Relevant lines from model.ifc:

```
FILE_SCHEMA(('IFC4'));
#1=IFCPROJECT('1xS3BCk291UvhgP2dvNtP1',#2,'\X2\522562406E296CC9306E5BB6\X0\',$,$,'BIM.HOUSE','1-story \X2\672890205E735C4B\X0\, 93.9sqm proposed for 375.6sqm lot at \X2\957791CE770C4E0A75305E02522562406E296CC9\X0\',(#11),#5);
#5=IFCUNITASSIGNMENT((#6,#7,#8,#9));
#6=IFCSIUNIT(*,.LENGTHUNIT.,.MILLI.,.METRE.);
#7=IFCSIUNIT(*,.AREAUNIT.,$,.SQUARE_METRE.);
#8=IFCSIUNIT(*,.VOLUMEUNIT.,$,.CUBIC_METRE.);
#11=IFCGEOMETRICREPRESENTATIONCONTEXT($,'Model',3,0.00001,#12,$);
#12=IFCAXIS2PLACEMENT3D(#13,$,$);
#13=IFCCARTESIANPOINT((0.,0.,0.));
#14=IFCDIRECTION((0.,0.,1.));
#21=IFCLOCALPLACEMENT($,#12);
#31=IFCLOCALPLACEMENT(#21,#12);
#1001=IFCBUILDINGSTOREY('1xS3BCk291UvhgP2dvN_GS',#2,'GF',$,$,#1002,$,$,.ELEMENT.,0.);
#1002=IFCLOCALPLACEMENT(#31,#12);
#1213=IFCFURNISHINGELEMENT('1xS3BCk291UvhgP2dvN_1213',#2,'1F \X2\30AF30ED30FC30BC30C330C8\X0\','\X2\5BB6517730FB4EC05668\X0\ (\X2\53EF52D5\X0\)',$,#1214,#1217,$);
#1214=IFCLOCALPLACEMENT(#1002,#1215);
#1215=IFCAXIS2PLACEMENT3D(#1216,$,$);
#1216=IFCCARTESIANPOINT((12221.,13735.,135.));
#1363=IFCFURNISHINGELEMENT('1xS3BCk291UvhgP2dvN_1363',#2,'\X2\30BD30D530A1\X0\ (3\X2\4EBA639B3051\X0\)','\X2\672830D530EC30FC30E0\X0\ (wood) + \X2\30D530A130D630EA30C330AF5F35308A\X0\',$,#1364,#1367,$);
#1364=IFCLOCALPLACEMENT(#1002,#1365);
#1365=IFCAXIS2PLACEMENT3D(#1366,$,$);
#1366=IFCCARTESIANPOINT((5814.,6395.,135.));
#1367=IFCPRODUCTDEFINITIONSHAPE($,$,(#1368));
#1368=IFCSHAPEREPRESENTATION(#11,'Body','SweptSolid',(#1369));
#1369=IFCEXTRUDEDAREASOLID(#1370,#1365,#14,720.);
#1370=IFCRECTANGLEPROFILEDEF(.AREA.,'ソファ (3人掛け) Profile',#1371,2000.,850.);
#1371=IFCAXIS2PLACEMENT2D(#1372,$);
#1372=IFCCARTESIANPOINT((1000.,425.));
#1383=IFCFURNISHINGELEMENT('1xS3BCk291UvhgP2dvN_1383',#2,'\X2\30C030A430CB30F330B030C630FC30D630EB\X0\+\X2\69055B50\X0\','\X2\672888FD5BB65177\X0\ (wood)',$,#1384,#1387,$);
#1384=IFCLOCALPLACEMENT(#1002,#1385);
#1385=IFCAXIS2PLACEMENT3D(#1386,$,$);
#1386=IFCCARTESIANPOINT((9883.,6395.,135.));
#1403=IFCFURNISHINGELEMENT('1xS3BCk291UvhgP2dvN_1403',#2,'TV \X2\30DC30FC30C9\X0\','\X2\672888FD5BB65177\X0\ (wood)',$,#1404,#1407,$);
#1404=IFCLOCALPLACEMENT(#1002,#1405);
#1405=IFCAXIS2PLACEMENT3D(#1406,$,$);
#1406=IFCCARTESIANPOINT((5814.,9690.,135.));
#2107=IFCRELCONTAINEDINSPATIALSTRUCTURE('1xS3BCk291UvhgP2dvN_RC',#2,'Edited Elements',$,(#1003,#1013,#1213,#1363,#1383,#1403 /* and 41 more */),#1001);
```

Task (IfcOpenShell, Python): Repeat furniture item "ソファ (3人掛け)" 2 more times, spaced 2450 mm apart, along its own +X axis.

```python
import ifcopenshell
import ifcopenshell.api.geometry
import ifcopenshell.api.root
import ifcopenshell.util.element
import ifcopenshell.util.placement
import ifcopenshell.util.unit

model = ifcopenshell.open("model.ifc")
unit_scale = ifcopenshell.util.unit.calculate_unit_scale(model)


def reuse_history(source, copy):
    """copy_class also copies each property set's owner history, people and application; keep the originals."""
    for rel in copy.IsDefinedBy:
        if rel.is_a("IfcRelDefinesByProperties") and (history := rel.RelatingPropertyDefinition.OwnerHistory):
            rel.RelatingPropertyDefinition.OwnerHistory = source.OwnerHistory
            ifcopenshell.util.element.remove_deep2(model, history)


source = model.by_id(1363)
base = ifcopenshell.util.placement.get_local_placement(source.ObjectPlacement)
step = base[:3, 0] * 2.45 / unit_scale

for i in range(1, 3):
    copy = ifcopenshell.api.root.copy_class(model, product=source)
    copy.Representation = ifcopenshell.util.element.copy_deep(
        model, source.Representation, exclude=["IfcGeometricRepresentationContext", "IfcRepresentationMap"]
    )
    reuse_history(source, copy)
    matrix = base.copy()
    matrix[:3, 3] += i * step
    print("added at", matrix[:3, 3].round(3) + 0.0)
    ifcopenshell.api.geometry.edit_object_placement(model, product=copy, matrix=matrix, is_si=False)

model.write("model_rev.ifc")
```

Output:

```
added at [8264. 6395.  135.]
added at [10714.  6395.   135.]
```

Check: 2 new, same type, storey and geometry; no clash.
